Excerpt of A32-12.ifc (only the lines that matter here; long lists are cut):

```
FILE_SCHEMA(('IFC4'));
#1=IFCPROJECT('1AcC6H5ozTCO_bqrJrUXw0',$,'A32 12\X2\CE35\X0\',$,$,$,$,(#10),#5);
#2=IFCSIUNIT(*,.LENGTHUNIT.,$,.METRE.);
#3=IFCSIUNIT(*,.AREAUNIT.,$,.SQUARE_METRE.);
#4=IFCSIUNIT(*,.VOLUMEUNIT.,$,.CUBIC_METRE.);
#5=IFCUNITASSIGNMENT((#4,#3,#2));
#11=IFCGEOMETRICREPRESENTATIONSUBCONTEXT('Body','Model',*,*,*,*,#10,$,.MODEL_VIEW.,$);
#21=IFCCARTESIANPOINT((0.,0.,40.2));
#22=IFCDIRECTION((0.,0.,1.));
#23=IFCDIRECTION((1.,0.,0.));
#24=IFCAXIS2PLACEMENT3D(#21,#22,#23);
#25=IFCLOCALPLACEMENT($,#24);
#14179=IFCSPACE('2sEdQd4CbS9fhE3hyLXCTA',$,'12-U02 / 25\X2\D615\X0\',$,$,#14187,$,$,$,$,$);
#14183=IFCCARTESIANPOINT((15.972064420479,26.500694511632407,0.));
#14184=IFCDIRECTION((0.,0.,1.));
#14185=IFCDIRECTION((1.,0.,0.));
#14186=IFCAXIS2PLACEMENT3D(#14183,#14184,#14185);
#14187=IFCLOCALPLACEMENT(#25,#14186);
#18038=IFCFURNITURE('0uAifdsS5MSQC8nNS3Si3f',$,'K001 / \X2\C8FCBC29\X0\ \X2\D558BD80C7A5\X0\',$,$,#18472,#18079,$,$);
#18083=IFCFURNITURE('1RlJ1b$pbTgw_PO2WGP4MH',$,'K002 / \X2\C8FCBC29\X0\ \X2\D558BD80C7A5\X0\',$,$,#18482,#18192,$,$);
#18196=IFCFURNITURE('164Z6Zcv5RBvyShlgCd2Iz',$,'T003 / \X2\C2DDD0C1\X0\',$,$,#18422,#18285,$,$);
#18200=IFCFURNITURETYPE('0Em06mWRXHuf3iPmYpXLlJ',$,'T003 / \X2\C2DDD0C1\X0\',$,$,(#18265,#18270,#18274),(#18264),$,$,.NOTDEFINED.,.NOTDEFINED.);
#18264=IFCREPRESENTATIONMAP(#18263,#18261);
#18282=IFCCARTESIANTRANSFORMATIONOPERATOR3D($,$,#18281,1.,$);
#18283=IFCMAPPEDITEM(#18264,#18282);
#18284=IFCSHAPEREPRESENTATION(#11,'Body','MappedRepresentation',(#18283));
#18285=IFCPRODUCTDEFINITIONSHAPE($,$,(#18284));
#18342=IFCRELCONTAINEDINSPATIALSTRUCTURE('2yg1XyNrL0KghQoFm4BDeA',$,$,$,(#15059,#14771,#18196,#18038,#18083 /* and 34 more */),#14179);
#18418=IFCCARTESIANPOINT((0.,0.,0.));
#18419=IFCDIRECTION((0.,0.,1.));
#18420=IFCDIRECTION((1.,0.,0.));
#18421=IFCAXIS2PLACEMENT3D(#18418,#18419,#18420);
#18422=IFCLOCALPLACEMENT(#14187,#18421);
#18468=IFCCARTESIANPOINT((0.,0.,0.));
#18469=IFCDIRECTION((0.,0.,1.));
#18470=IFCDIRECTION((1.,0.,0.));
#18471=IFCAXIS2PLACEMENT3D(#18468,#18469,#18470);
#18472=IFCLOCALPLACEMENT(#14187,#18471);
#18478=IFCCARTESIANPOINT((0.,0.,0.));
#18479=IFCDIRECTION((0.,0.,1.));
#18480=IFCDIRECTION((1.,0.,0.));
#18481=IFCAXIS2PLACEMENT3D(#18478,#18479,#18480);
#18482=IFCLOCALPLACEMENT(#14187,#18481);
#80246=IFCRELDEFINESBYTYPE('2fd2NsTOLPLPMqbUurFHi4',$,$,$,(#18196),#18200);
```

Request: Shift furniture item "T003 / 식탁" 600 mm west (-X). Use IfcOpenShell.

```python
import ifcopenshell
import ifcopenshell.api.geometry
import ifcopenshell.util.placement

model = ifcopenshell.open("A32-12.ifc")

item = model.by_guid("164Z6Zcv5RBvyShlgCd2Iz")
matrix = ifcopenshell.util.placement.get_local_placement(item.ObjectPlacement)
matrix[0, 3] -= 0.6
ifcopenshell.api.geometry.edit_object_placement(model, product=item, matrix=matrix, is_si=False)

print(ifcopenshell.util.placement.get_local_placement(item.ObjectPlacement).round(3) + 0.0)

model.write("A32-12_rev.ifc")
```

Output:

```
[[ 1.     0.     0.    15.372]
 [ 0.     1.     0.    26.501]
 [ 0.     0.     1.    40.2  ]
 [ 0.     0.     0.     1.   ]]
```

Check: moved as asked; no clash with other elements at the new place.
